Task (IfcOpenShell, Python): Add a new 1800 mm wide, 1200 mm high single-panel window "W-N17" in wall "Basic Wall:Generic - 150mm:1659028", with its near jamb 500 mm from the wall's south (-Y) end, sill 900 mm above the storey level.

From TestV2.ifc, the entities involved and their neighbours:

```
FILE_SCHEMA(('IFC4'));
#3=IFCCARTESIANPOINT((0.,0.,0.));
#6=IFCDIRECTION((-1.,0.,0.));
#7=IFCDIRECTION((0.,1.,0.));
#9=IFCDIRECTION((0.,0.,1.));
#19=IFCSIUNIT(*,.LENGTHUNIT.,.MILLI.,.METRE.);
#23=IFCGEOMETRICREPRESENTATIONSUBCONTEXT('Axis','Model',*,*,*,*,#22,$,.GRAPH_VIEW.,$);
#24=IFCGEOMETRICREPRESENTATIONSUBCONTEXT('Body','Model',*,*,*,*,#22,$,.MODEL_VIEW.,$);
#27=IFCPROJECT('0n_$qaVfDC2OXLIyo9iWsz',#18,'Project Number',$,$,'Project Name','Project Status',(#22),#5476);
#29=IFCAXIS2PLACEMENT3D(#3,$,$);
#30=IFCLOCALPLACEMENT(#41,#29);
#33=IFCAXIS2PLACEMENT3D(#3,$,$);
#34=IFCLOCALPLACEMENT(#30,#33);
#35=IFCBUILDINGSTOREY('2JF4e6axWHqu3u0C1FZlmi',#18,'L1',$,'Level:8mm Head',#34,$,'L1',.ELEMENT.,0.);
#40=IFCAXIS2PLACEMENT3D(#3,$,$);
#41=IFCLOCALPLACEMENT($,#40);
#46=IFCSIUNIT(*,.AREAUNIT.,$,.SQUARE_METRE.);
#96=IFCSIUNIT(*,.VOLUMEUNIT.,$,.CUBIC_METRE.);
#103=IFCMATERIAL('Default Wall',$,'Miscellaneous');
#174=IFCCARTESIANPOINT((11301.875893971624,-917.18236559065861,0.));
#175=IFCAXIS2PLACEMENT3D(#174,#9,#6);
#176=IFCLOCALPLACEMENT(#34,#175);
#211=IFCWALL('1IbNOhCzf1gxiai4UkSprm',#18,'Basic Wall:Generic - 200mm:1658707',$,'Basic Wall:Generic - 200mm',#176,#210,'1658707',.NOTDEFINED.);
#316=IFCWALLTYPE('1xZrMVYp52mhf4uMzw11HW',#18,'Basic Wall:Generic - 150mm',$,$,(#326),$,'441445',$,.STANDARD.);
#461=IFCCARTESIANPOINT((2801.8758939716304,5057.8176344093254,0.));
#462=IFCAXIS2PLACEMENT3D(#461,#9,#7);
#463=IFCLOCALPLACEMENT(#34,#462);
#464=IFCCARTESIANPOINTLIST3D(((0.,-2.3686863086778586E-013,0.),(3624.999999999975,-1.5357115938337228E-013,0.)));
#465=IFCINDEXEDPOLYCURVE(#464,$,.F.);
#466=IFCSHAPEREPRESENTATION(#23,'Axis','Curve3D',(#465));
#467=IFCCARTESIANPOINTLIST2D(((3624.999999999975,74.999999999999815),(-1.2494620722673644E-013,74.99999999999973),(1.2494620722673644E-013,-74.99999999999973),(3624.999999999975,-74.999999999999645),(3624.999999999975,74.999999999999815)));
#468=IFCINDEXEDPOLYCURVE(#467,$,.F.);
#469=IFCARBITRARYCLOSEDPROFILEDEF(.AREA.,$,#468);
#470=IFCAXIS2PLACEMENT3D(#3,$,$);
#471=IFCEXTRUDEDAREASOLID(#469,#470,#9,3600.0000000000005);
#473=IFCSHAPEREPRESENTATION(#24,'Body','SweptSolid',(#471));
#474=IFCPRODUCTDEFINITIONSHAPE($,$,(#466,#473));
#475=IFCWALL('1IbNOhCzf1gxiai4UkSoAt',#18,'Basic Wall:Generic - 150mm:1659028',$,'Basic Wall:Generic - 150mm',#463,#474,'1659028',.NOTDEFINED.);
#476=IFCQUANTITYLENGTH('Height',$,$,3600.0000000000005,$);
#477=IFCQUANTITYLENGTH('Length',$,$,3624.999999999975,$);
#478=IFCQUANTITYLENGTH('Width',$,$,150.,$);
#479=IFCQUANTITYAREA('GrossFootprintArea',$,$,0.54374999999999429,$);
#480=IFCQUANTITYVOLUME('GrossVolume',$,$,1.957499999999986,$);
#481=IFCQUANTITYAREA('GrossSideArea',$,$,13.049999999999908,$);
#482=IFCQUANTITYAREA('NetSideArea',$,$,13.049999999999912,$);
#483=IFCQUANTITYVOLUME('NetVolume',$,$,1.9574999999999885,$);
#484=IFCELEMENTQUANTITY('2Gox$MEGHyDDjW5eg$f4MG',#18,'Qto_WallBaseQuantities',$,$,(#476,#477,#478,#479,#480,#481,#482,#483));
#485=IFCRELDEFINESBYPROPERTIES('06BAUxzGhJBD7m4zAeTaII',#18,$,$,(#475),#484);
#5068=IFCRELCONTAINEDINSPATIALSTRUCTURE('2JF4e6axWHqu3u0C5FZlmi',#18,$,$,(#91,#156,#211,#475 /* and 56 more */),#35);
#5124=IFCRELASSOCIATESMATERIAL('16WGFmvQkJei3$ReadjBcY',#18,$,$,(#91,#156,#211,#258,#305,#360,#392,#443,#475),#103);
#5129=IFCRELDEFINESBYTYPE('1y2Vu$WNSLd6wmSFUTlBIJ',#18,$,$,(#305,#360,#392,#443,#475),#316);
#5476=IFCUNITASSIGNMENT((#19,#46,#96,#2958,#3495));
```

```python
import numpy as np
import ifcopenshell
import ifcopenshell.api.feature
import ifcopenshell.api.geometry
import ifcopenshell.api.pset
import ifcopenshell.api.root
import ifcopenshell.api.spatial
import ifcopenshell.geom
import ifcopenshell.util.element
import ifcopenshell.util.placement
import ifcopenshell.util.representation
import ifcopenshell.util.shape
import ifcopenshell.util.unit

model = ifcopenshell.open("TestV2.ifc")
unit_scale = ifcopenshell.util.unit.calculate_unit_scale(model)
area_scale = ifcopenshell.util.unit.calculate_unit_scale(model, "AREAUNIT")
volume_scale = ifcopenshell.util.unit.calculate_unit_scale(model, "VOLUMEUNIT")
settings = ifcopenshell.geom.settings()


def volume(element):
    """Net volume in cubic metres, openings subtracted."""
    shape = ifcopenshell.geom.create_shape(settings, element)
    return ifcopenshell.util.shape.get_volume(shape.geometry)


wall = model.by_guid("1IbNOhCzf1gxiai4UkSoAt")
storey = ifcopenshell.util.element.get_container(wall, ifc_class="IfcBuildingStorey")
context = ifcopenshell.util.representation.get_context(model, "Model", "Body", "MODEL_VIEW")
before = volume(wall)

width, height, from_end, sill = 1.8, 1.2, 0.5, 0.9  # metres

# The wall runs along its own X axis, and the end named is its -X end.
wall_shape = ifcopenshell.geom.create_shape(settings, wall)
x, y, z = ifcopenshell.util.shape.get_vertices(wall_shape.geometry).T
start = x.min() + from_end
face, thickness = float(y.min()), float(y.max() - y.min())
wall_matrix = ifcopenshell.util.placement.get_local_placement(wall.ObjectPlacement)
level = ifcopenshell.util.placement.get_local_placement(storey.ObjectPlacement)[2, 3]


def in_wall(x, y):
    """Placement at x, y metres in the wall's axes, at sill height."""
    matrix = wall_matrix.copy()
    matrix[:, 3] = wall_matrix @ np.array([x / unit_scale, y / unit_scale, 0.0, 1.0])
    matrix[2, 3] = level + sill / unit_scale
    return matrix


# Opening: a box that overshoots both wall faces by 50 mm.
opening = ifcopenshell.api.root.create_entity(model, ifc_class="IfcOpeningElement", predefined_type="OPENING")
box = ifcopenshell.api.geometry.add_wall_representation(
    model, context=context, length=width, height=height, thickness=thickness + 0.1
)
ifcopenshell.api.geometry.assign_representation(model, product=opening, representation=box)
ifcopenshell.api.geometry.edit_object_placement(model, product=opening, matrix=in_wall(start, face - 0.05), is_si=False)
ifcopenshell.api.feature.add_feature(model, feature=opening, element=wall)

window = ifcopenshell.api.root.create_entity(model, ifc_class="IfcWindow", name="W-N17", predefined_type="WINDOW")
window.OverallWidth, window.OverallHeight = width / unit_scale, height / unit_scale
window.PartitioningType = "SINGLE_PANEL"
body = ifcopenshell.api.geometry.add_window_representation(
    model,
    context=context,
    overall_width=window.OverallWidth,
    overall_height=window.OverallHeight,
    partition_type="SINGLE_PANEL",
)
ifcopenshell.api.geometry.assign_representation(model, product=window, representation=body)
ifcopenshell.api.spatial.assign_container(model, products=[window], relating_structure=storey)
ifcopenshell.api.feature.add_filling(model, opening=opening, element=window)

# Centre the window in the wall's thickness.
ifcopenshell.api.geometry.edit_object_placement(model, product=window, matrix=in_wall(start, face), is_si=False)
window_shape = ifcopenshell.geom.create_shape(settings, window)
depth = ifcopenshell.util.shape.get_vertices(window_shape.geometry)[:, 1]
offset = face + thickness / 2 - (depth.min() + depth.max()) / 2
ifcopenshell.api.geometry.edit_object_placement(model, product=window, matrix=in_wall(start, offset), is_si=False)

after = volume(wall)

# Update the wall's stored quantities.
qto = model.by_id(ifcopenshell.util.element.get_pset(wall, "Qto_WallBaseQuantities", should_inherit=False)["id"])
ifcopenshell.api.pset.edit_qto(model, qto=qto, properties={
    "NetSideArea": after / thickness / area_scale,
    "NetVolume": after / volume_scale,
})

print(f"wall volume {before:.3f} -> {after:.3f} m3")

model.write("TestV2_rev.ifc")
```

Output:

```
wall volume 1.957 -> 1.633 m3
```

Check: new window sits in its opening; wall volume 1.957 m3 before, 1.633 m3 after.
